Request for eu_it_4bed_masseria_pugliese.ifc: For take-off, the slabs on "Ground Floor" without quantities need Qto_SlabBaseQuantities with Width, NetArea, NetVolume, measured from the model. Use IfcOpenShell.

First a look at what the model holds.

```python
import ifcopenshell
import ifcopenshell.util.element
import ifcopenshell.util.unit

model = ifcopenshell.open("eu_it_4bed_masseria_pugliese.ifc")
print(model.schema)
for unit_type in ("LENGTHUNIT", "AREAUNIT", "VOLUMEUNIT"):
    print(unit_type, ifcopenshell.util.unit.calculate_unit_scale(model, unit_type))
storey = next(s for s in model.by_type("IfcBuildingStorey") if s.Name == "Ground Floor")
slabs = [e for e in ifcopenshell.util.element.get_decomposition(storey) if e.is_a("IfcSlab")]
for e in sorted(slabs, key=lambda e: e.id()):
    print(e.id(), e.is_a(), e.Name, list(ifcopenshell.util.element.get_psets(e, qtos_only=True)), sep=" | ")
```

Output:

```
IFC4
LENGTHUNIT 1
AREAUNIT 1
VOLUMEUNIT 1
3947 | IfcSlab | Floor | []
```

```python
import ifcopenshell
import ifcopenshell.api.pset
import ifcopenshell.geom
import ifcopenshell.util.element
import ifcopenshell.util.shape
import ifcopenshell.util.unit

model = ifcopenshell.open("eu_it_4bed_masseria_pugliese.ifc")
unit_scale = ifcopenshell.util.unit.calculate_unit_scale(model)
area_scale = ifcopenshell.util.unit.calculate_unit_scale(model, "AREAUNIT")
volume_scale = ifcopenshell.util.unit.calculate_unit_scale(model, "VOLUMEUNIT")
settings = ifcopenshell.geom.settings()

storey = next(s for s in model.by_type("IfcBuildingStorey") if s.Name == "Ground Floor")
slabs = [e for e in ifcopenshell.util.element.get_decomposition(storey) if e.is_a("IfcSlab")]

for e in sorted(slabs, key=lambda e: e.id()):
    if ifcopenshell.util.element.get_psets(e, qtos_only=True, should_inherit=False):
        continue
    # Geometry comes back in metres, in the element's own axes.
    shape = ifcopenshell.geom.create_shape(settings, e)
    values = {
        "Width": ifcopenshell.util.shape.get_z(shape.geometry) / unit_scale,
        "NetArea": ifcopenshell.util.shape.get_footprint_area(shape.geometry) / area_scale,
        "NetVolume": ifcopenshell.util.shape.get_volume(shape.geometry) / volume_scale,
    }
    qto = ifcopenshell.api.pset.add_qto(model, product=e, name="Qto_SlabBaseQuantities")
    ifcopenshell.api.pset.edit_qto(model, qto=qto, properties=values)
    print(e.id(), {k: round(v, 3) for k, v in values.items()})

model.write("eu_it_4bed_masseria_pugliese_edited.ifc")
```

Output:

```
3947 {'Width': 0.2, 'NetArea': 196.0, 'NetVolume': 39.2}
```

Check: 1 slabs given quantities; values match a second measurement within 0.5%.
